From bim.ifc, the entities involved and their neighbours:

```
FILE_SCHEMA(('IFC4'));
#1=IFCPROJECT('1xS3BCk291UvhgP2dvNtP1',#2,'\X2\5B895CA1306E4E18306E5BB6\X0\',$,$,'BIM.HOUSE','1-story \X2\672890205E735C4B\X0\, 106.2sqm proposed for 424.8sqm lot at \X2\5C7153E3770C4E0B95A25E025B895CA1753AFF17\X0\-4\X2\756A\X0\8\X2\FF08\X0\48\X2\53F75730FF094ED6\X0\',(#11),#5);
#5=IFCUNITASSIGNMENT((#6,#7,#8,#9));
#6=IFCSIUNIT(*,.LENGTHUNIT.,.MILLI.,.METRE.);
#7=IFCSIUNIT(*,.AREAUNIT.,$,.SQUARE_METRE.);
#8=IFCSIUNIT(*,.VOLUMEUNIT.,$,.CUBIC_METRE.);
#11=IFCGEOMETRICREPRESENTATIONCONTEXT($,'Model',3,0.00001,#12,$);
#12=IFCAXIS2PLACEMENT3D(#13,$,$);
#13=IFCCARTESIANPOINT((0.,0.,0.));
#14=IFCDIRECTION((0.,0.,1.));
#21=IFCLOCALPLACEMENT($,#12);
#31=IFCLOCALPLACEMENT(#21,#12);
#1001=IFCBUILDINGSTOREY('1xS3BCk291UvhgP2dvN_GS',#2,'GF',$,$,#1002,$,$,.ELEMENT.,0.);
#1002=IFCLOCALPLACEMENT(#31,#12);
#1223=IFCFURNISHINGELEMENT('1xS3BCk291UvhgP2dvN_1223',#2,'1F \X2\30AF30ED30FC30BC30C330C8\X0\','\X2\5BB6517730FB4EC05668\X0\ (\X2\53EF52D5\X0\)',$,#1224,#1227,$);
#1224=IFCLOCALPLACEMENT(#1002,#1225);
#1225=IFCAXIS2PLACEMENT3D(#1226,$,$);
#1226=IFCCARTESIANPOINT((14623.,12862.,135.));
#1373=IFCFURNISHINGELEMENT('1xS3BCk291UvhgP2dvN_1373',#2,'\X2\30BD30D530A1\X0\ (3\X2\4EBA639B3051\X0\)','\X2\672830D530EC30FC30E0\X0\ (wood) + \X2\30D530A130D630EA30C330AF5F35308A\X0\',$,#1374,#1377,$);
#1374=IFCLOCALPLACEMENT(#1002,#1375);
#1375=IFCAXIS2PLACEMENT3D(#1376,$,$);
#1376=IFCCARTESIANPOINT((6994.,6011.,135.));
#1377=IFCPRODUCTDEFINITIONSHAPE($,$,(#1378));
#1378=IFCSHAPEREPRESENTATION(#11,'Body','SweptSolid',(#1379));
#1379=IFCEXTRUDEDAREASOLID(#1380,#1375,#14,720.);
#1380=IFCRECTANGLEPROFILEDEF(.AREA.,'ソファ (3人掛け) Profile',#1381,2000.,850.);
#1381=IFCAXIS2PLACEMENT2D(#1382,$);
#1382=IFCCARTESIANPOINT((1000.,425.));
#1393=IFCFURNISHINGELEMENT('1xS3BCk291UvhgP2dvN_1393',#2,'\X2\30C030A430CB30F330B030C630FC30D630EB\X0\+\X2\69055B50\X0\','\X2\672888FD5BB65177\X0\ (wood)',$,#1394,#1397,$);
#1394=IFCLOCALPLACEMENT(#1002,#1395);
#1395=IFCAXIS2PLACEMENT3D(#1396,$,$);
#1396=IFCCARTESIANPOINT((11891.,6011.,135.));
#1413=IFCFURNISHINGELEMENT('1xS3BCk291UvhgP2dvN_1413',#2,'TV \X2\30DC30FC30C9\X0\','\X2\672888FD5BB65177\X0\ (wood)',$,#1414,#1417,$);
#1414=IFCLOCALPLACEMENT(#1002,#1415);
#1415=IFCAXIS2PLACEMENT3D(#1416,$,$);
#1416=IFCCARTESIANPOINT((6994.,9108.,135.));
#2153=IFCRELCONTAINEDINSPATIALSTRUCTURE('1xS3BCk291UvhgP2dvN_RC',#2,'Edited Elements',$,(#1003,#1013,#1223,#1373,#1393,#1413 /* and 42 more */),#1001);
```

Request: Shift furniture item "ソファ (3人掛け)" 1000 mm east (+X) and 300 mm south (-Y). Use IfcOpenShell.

```python
import ifcopenshell
import ifcopenshell.api.geometry
import ifcopenshell.util.placement

model = ifcopenshell.open("bim.ifc")

item = model.by_guid("1xS3BCk291UvhgP2dvN_1373")
matrix = ifcopenshell.util.placement.get_local_placement(item.ObjectPlacement)
matrix[0, 3] += 1000.0
matrix[1, 3] -= 300.0
ifcopenshell.api.geometry.edit_object_placement(model, product=item, matrix=matrix, is_si=False)

print(ifcopenshell.util.placement.get_local_placement(item.ObjectPlacement).round(3) + 0.0)

model.write("bim_rev.ifc")
```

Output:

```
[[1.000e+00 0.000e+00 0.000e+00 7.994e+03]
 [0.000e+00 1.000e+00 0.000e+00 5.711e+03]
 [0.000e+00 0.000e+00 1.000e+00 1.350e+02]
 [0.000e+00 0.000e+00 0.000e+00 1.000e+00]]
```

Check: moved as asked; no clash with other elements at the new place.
